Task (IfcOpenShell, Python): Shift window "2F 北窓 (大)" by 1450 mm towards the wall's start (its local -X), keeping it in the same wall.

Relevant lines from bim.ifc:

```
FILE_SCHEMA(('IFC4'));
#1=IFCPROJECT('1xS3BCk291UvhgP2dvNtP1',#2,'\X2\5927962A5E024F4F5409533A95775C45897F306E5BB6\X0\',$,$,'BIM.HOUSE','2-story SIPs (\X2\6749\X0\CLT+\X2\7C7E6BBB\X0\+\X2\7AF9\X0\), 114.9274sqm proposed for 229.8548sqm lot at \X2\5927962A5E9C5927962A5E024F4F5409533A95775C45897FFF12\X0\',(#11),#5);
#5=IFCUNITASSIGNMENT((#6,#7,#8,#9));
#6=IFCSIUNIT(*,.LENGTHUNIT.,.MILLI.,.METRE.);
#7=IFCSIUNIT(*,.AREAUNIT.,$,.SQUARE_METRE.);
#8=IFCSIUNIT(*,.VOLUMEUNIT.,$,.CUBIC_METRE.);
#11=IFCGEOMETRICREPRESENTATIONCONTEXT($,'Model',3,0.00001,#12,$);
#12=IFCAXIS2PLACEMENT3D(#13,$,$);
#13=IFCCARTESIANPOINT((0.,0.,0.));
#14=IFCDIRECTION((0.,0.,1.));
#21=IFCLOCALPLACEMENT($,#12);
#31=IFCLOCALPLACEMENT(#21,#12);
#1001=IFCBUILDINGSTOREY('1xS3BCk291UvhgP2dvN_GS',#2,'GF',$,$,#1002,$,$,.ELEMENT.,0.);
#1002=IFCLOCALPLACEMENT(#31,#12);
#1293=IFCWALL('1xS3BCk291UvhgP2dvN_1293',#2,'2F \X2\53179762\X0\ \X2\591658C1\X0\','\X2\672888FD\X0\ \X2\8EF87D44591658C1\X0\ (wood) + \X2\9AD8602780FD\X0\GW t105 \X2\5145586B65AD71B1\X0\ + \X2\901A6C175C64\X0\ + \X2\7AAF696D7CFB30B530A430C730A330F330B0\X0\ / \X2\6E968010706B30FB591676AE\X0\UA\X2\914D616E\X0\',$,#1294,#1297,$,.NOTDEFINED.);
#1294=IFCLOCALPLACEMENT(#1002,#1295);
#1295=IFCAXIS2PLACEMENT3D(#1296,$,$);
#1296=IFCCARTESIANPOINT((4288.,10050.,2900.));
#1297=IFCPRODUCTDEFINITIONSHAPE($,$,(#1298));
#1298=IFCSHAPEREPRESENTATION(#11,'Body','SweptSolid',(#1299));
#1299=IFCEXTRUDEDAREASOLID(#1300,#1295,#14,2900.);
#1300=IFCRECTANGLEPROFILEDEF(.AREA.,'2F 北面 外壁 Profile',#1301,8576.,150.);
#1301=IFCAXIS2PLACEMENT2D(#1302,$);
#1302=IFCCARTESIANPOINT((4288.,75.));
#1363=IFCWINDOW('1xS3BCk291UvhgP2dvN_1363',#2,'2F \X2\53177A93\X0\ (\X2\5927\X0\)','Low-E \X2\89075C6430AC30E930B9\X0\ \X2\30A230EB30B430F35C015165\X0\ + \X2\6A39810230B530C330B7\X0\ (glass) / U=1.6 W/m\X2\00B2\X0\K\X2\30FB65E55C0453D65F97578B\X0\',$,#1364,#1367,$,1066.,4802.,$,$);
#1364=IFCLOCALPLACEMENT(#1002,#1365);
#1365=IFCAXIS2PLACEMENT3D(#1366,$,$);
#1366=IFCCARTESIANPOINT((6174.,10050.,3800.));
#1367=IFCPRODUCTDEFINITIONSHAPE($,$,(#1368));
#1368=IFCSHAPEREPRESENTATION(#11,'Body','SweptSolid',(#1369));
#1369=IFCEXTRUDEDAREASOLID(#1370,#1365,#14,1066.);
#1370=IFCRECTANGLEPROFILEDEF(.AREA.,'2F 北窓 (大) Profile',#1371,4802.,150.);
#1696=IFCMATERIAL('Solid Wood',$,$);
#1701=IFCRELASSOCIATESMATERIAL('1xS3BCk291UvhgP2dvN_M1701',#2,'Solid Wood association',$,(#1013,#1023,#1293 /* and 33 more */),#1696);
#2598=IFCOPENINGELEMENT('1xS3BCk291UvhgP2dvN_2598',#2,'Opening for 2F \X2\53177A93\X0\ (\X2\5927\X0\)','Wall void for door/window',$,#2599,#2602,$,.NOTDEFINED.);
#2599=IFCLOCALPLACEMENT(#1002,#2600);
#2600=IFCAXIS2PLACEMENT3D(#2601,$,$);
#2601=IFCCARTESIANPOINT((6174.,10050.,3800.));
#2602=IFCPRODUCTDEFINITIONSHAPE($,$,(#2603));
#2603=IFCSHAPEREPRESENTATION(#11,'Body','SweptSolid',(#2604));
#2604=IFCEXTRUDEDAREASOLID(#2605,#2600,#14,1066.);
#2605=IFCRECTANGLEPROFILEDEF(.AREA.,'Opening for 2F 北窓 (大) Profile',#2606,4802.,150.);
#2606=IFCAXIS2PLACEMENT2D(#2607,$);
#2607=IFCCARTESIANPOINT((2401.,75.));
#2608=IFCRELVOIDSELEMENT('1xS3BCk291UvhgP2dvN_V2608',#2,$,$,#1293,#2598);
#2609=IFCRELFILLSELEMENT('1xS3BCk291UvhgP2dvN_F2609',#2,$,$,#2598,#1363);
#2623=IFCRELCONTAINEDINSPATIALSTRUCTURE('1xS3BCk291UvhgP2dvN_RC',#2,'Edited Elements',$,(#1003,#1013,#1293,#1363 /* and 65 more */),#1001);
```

```python
import ifcopenshell
import ifcopenshell.api.geometry
import ifcopenshell.util.placement
import ifcopenshell.util.unit

model = ifcopenshell.open("bim.ifc")
unit_scale = ifcopenshell.util.unit.calculate_unit_scale(model)

window = model.by_guid("1xS3BCk291UvhgP2dvN_1363")
opening = window.FillsVoids[0].RelatingOpeningElement
wall = opening.VoidsElements[0].RelatingBuildingElement

wall_matrix = ifcopenshell.util.placement.get_local_placement(wall.ObjectPlacement)
shift = wall_matrix[:3, 0] * -1.45 / unit_scale
before = ifcopenshell.util.placement.get_local_placement(window.ObjectPlacement)[:3, 3].copy()

# The window is not placed relative to its opening, so move both.
for product in (opening, window):
    matrix = ifcopenshell.util.placement.get_local_placement(product.ObjectPlacement)
    matrix[:3, 3] += shift
    ifcopenshell.api.geometry.edit_object_placement(model, product=product, matrix=matrix, is_si=False)

after = ifcopenshell.util.placement.get_local_placement(window.ObjectPlacement)[:3, 3]
print("window moved by", (after - before).round(3) + 0.0)

model.write("bim_v2.ifc")
```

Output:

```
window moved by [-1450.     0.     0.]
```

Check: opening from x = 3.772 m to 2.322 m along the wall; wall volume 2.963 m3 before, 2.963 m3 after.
